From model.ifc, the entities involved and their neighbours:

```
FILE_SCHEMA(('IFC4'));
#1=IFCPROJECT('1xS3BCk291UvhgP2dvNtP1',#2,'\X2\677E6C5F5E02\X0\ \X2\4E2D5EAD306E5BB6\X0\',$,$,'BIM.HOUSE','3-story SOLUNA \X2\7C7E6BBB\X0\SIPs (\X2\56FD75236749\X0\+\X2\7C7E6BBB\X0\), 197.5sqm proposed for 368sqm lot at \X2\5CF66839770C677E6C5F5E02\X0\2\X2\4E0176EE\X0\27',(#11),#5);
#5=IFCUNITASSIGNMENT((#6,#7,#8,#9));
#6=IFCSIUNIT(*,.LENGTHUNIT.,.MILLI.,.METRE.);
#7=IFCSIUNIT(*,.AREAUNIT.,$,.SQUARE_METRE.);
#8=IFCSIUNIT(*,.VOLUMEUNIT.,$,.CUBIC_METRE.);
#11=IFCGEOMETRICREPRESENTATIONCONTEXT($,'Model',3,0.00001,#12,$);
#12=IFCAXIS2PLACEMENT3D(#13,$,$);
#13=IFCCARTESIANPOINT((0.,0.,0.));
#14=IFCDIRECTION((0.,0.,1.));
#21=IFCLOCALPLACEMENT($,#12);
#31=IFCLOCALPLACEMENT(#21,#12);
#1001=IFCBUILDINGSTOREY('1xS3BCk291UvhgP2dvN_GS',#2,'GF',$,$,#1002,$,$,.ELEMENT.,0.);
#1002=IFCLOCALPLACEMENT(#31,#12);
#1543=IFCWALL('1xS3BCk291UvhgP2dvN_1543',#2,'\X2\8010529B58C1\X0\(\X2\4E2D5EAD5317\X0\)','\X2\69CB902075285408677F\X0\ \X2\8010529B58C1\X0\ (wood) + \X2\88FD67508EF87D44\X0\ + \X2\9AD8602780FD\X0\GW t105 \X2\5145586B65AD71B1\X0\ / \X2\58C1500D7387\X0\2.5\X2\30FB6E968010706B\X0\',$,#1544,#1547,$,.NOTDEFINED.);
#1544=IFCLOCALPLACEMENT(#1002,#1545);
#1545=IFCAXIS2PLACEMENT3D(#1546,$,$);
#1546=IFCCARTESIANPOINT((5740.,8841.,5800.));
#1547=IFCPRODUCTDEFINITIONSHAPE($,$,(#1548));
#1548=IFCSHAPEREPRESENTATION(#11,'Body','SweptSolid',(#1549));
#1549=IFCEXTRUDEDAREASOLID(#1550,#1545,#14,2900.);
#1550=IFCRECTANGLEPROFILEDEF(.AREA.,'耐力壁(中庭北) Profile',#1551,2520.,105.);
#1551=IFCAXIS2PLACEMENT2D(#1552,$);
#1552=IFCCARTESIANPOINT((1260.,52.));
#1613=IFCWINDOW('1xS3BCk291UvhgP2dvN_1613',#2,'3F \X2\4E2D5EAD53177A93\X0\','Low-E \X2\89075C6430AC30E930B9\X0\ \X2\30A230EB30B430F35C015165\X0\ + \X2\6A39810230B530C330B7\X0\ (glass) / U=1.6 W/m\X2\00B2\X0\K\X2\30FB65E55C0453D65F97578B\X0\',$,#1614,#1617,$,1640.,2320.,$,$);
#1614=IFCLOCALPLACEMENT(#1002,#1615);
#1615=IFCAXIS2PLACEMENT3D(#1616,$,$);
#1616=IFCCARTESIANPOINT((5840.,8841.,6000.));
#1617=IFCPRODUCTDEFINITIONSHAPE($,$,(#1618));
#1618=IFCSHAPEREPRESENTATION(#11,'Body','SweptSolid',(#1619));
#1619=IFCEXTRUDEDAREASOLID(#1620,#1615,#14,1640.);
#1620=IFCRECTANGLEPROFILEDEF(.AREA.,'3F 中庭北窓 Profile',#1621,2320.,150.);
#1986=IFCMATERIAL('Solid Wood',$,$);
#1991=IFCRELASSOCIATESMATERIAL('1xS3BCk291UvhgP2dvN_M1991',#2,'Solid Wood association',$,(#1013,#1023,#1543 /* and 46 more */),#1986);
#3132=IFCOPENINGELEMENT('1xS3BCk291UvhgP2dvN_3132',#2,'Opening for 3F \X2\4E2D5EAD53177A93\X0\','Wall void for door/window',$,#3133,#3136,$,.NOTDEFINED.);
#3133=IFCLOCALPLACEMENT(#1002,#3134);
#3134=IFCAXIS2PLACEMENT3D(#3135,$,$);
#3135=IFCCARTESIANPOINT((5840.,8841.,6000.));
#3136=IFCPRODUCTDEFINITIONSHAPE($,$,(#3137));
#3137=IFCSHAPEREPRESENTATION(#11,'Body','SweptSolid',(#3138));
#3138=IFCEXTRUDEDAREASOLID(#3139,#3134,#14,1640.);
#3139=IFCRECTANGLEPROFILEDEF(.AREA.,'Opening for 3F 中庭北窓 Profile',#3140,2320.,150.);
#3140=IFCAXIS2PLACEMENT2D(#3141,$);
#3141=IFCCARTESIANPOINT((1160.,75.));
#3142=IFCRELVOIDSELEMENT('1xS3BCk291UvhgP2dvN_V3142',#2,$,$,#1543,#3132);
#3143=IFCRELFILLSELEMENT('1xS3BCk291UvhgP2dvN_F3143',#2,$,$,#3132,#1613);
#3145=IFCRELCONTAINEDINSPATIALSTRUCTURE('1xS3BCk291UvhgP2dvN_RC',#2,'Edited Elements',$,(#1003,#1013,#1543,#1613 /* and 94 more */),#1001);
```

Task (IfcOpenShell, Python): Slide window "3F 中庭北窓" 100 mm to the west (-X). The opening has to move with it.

```python
import ifcopenshell
import ifcopenshell.api.geometry
import ifcopenshell.util.placement
import ifcopenshell.util.unit

model = ifcopenshell.open("model.ifc")
unit_scale = ifcopenshell.util.unit.calculate_unit_scale(model)

window = model.by_guid("1xS3BCk291UvhgP2dvN_1613")
opening = window.FillsVoids[0].RelatingOpeningElement
wall = opening.VoidsElements[0].RelatingBuildingElement

wall_matrix = ifcopenshell.util.placement.get_local_placement(wall.ObjectPlacement)
shift = wall_matrix[:3, 0] * -0.1 / unit_scale
before = ifcopenshell.util.placement.get_local_placement(window.ObjectPlacement)[:3, 3].copy()

# The window is not placed relative to its opening, so move both.
for product in (opening, window):
    matrix = ifcopenshell.util.placement.get_local_placement(product.ObjectPlacement)
    matrix[:3, 3] += shift
    ifcopenshell.api.geometry.edit_object_placement(model, product=product, matrix=matrix, is_si=False)

after = ifcopenshell.util.placement.get_local_placement(window.ObjectPlacement)[:3, 3]
print("window moved by", (after - before).round(3) + 0.0)

model.write("model_edited.ifc")
```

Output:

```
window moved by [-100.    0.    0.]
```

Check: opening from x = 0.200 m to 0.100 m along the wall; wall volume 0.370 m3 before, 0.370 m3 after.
